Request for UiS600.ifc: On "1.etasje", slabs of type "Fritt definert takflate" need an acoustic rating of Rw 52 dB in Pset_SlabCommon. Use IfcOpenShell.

First a look at what the model holds.

```python
import ifcopenshell
import ifcopenshell.util.element

model = ifcopenshell.open("UiS600.ifc")
print(model.schema)
storey = next(s for s in model.by_type("IfcBuildingStorey") if s.Name == "1.etasje")
slabs = [e for e in ifcopenshell.util.element.get_decomposition(storey) if e.is_a("IfcSlab")]
seen = {}
for e in slabs:
    element_type = ifcopenshell.util.element.get_type(e)
    key = (element_type.Name if element_type != e and element_type else None, ifcopenshell.util.element.get_pset(e, "Pset_SlabCommon", "AcousticRating"))
    seen[key] = seen.get(key, 0) + 1
for (name, value), count in sorted(seen.items(), key=str):
    print(count, "x", name, "|", value)
```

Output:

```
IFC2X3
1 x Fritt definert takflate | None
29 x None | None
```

```python
import ifcopenshell
import ifcopenshell.api.pset
import ifcopenshell.util.element

model = ifcopenshell.open("UiS600.ifc")

storey = next(s for s in model.by_type("IfcBuildingStorey") if s.Name == "1.etasje")
slabs = [e for e in ifcopenshell.util.element.get_decomposition(storey) if e.is_a("IfcSlab")]

count = 0
for e in slabs:
    element_type = ifcopenshell.util.element.get_type(e)
    if element_type in (None, e) or element_type.Name != "Fritt definert takflate":
        continue
    # add_pset returns the element's existing set when there is one.
    pset = ifcopenshell.api.pset.add_pset(model, product=e, name="Pset_SlabCommon")
    ifcopenshell.api.pset.edit_pset(model, pset=pset, properties={"AcousticRating": "Rw 52 dB"})
    count += 1

print(count, "slabs updated")

model.write("UiS600_updated.ifc")
```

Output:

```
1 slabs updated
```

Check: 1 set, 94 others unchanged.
